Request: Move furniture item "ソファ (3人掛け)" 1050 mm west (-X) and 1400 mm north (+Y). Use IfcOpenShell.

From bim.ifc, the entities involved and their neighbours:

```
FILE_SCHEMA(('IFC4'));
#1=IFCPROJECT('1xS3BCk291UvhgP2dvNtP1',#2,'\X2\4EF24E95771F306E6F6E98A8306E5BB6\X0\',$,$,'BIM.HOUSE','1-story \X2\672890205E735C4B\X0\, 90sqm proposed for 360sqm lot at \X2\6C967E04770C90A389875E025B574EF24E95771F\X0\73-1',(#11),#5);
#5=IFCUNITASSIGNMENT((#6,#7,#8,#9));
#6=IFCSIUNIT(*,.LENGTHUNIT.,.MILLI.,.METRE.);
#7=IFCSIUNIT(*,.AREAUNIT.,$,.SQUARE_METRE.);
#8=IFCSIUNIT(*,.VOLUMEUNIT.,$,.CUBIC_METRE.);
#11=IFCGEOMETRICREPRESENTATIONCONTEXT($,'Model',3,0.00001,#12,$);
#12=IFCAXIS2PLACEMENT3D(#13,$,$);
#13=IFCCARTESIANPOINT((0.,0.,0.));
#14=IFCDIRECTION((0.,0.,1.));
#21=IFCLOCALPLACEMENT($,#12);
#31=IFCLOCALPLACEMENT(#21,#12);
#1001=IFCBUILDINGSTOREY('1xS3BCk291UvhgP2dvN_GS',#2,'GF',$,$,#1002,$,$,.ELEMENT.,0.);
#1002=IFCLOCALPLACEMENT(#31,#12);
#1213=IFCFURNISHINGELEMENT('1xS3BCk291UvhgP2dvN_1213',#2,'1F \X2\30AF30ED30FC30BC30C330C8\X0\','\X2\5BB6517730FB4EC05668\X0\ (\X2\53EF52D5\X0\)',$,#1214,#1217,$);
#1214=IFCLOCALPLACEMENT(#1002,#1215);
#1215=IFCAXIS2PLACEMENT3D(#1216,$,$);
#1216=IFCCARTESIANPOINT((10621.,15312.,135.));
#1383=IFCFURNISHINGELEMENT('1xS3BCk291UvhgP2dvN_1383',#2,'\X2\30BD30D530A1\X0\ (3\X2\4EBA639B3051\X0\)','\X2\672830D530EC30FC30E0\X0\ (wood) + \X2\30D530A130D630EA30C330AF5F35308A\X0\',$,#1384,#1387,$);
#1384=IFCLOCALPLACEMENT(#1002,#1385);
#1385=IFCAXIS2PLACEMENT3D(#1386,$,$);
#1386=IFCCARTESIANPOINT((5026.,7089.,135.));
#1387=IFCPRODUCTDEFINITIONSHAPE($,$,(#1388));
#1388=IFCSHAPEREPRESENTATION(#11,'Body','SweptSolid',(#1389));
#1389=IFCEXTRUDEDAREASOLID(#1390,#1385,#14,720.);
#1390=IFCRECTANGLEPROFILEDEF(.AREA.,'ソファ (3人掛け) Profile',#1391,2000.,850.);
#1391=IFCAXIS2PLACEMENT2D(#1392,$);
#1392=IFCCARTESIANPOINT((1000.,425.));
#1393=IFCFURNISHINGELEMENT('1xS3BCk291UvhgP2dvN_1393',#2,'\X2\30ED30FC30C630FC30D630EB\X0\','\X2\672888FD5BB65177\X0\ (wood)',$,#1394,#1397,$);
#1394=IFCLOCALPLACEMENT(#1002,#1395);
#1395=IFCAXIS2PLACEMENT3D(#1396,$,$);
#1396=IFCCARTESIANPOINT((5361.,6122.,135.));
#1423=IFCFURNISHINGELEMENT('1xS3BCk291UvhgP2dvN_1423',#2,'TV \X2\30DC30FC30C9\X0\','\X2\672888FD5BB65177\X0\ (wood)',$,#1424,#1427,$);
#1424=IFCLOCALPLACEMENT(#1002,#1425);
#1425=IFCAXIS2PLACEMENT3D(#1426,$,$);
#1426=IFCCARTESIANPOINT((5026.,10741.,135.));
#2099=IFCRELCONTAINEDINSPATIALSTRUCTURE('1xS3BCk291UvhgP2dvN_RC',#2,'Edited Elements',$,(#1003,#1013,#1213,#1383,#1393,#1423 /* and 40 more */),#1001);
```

```python
import ifcopenshell
import ifcopenshell.api.geometry
import ifcopenshell.util.placement

model = ifcopenshell.open("bim.ifc")

item = model.by_guid("1xS3BCk291UvhgP2dvN_1383")
matrix = ifcopenshell.util.placement.get_local_placement(item.ObjectPlacement)
matrix[0, 3] -= 1050.0
matrix[1, 3] += 1400.0
ifcopenshell.api.geometry.edit_object_placement(model, product=item, matrix=matrix, is_si=False)

print(ifcopenshell.util.placement.get_local_placement(item.ObjectPlacement).round(3) + 0.0)

model.write("bim_rev.ifc")
```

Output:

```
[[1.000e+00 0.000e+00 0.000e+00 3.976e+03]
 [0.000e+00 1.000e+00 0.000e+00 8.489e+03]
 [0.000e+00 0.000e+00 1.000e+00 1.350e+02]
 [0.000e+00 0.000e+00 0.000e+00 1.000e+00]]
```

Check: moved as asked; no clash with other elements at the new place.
